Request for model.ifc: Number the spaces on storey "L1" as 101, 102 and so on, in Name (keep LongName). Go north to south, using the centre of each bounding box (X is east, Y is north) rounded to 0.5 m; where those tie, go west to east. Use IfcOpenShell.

First a look at what the model holds.

```python
import ifcopenshell
import ifcopenshell.util.element
import ifcopenshell.util.placement

model = ifcopenshell.open("model.ifc")
print(model.schema)
storey = next(s for s in model.by_type("IfcBuildingStorey") if s.Name == "L1")
spaces = [e for e in ifcopenshell.util.element.get_decomposition(storey) if e.is_a("IfcSpace")]
for e in sorted(spaces, key=lambda e: e.id()):
    origin = ifcopenshell.util.placement.get_local_placement(e.ObjectPlacement)[:3, 3]
    print(e.id(), e.Name, e.LongName, origin.round(2) + 0.0, sep=" | ")
```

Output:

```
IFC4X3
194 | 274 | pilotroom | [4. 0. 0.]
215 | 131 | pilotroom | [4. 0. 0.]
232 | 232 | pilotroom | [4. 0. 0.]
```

```python
import ifcopenshell
import ifcopenshell.geom
import ifcopenshell.util.element
import ifcopenshell.util.shape

model = ifcopenshell.open("model.ifc")
settings = ifcopenshell.geom.settings()
settings.set("use-world-coords", True)


def centre(element):
    shape = ifcopenshell.geom.create_shape(settings, element)
    return ifcopenshell.util.shape.get_bbox_centroid(shape.geometry)


storey = next(s for s in model.by_type("IfcBuildingStorey") if s.Name == "L1")
spaces = [e for e in ifcopenshell.util.element.get_decomposition(storey) if e.is_a("IfcSpace")]

# Insertion points can sit at a corner or the storey origin, so sort by the geometry (in metres).
centres = {e: centre(e) for e in spaces}
spaces.sort(key=lambda e: (-round(centres[e][1] / 0.5), centres[e][0]))

for i, e in enumerate(spaces, start=1):
    number = f"1{i:02d}"
    e.Name = number
    print(e.id(), number)

model.write("model_v2.ifc")
```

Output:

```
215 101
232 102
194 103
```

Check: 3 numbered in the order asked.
